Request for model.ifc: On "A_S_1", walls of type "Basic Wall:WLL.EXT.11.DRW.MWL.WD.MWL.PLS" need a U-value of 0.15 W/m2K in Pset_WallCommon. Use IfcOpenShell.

First a look at what the model holds.

```python
import ifcopenshell
import ifcopenshell.util.element

model = ifcopenshell.open("model.ifc")
print(model.schema)
storey = next(s for s in model.by_type("IfcBuildingStorey") if s.Name == "A_S_1")
walls = [e for e in ifcopenshell.util.element.get_decomposition(storey) if e.is_a("IfcWall")]
seen = {}
for e in walls:
    element_type = ifcopenshell.util.element.get_type(e)
    key = (element_type.Name if element_type != e and element_type else None, ifcopenshell.util.element.get_pset(e, "Pset_WallCommon", "ThermalTransmittance"))
    seen[key] = seen.get(key, 0) + 1
for (name, value), count in sorted(seen.items(), key=str):
    print(count, "x", name, "|", value)
```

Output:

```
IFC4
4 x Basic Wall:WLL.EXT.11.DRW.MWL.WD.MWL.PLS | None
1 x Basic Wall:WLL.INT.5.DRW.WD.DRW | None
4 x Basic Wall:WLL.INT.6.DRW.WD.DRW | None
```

```python
import ifcopenshell
import ifcopenshell.api.pset
import ifcopenshell.util.element

model = ifcopenshell.open("model.ifc")

storey = next(s for s in model.by_type("IfcBuildingStorey") if s.Name == "A_S_1")
walls = [e for e in ifcopenshell.util.element.get_decomposition(storey) if e.is_a("IfcWall")]

count = 0
for e in walls:
    element_type = ifcopenshell.util.element.get_type(e)
    if element_type in (None, e) or element_type.Name != "Basic Wall:WLL.EXT.11.DRW.MWL.WD.MWL.PLS":
        continue
    # add_pset returns the element's existing set when there is one.
    pset = ifcopenshell.api.pset.add_pset(model, product=e, name="Pset_WallCommon")
    ifcopenshell.api.pset.edit_pset(model, pset=pset, properties={"ThermalTransmittance": 0.15})
    count += 1

print(count, "walls updated")

model.write("model_rev.ifc")
```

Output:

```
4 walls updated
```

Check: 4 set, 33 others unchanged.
